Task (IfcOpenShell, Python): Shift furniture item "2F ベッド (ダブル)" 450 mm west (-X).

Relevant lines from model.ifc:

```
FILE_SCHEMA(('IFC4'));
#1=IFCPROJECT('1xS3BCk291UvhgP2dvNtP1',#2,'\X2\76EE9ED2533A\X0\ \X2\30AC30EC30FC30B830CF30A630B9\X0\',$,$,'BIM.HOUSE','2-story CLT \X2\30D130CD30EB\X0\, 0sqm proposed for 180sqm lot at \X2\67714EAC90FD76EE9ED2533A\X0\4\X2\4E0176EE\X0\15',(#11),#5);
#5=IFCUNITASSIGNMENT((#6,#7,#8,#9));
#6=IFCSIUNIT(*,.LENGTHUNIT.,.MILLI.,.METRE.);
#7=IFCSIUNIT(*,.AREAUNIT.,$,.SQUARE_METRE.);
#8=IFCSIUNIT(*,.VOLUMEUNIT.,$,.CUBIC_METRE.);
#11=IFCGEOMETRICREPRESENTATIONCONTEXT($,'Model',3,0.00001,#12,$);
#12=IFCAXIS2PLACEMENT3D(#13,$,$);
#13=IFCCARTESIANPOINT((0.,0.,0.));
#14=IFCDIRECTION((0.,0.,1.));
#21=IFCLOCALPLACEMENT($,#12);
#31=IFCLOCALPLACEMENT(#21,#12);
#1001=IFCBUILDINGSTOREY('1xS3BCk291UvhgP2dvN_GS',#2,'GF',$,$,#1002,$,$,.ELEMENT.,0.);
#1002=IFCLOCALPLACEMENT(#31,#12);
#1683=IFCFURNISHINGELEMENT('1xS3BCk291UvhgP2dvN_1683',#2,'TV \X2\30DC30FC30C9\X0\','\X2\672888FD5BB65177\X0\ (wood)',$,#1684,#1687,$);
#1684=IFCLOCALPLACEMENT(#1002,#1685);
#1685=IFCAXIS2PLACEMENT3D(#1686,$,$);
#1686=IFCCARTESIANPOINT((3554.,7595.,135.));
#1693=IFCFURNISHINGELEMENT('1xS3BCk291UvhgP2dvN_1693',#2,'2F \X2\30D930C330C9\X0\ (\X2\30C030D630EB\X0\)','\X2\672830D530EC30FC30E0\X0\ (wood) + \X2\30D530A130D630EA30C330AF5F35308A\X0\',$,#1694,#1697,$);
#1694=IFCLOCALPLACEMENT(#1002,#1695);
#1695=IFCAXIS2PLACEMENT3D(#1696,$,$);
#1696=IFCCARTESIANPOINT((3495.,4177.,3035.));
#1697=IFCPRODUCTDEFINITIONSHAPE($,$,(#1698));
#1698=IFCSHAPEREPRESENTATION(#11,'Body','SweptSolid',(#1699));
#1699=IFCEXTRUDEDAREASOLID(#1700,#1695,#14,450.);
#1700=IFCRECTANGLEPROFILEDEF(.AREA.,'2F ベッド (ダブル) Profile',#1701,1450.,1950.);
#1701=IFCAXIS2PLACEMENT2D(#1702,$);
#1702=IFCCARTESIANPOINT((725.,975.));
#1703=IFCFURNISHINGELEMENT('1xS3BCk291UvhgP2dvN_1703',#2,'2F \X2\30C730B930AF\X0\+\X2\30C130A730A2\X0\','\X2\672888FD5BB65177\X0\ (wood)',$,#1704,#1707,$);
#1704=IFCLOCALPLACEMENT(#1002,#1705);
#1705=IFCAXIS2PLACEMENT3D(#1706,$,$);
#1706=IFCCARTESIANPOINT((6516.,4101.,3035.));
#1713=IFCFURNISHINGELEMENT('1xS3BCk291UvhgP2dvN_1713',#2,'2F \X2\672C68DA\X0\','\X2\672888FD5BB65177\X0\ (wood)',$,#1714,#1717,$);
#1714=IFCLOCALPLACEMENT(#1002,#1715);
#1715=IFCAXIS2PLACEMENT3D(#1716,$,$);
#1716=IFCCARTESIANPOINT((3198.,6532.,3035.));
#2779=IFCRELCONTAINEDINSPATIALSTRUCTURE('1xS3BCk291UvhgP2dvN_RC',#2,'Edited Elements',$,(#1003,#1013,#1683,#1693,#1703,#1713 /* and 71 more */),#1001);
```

```python
import ifcopenshell
import ifcopenshell.api.geometry
import ifcopenshell.util.placement

model = ifcopenshell.open("model.ifc")

item = model.by_guid("1xS3BCk291UvhgP2dvN_1693")
matrix = ifcopenshell.util.placement.get_local_placement(item.ObjectPlacement)
matrix[0, 3] -= 450.0
ifcopenshell.api.geometry.edit_object_placement(model, product=item, matrix=matrix, is_si=False)

print(ifcopenshell.util.placement.get_local_placement(item.ObjectPlacement).round(3) + 0.0)

model.write("model_updated.ifc")
```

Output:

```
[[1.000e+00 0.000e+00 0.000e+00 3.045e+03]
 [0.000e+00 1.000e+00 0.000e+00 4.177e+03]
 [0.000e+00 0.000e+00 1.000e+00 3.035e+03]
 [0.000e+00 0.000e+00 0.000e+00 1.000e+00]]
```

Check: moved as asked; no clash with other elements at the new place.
